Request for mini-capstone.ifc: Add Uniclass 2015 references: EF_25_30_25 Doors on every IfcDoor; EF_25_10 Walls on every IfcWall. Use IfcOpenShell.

First a look at what the model holds.

```python
import ifcopenshell

model = ifcopenshell.open("mini-capstone.ifc")
print(model.schema)
print("classifications:", [c.Name for c in model.by_type("IfcClassification")])
for ifc_class in ("IfcDoor", "IfcRoof", "IfcStair", "IfcWall", "IfcWindow"):
    print(ifc_class, len(model.by_type(ifc_class)))
```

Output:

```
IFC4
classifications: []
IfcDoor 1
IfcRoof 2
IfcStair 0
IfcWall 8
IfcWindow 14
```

```python
import ifcopenshell
import ifcopenshell.api.classification

model = ifcopenshell.open("mini-capstone.ifc")

system = ifcopenshell.api.classification.add_classification(model, classification="Uniclass 2015")

codes = {
    "IfcDoor": ("EF_25_30_25", "Doors"),
    "IfcWall": ("EF_25_10", "Walls"),
}
for ifc_class, (code, name) in codes.items():
    products = model.by_type(ifc_class)
    ifcopenshell.api.classification.add_reference(
        model, products=products, classification=system, identification=code, name=name
    )
    print(code, len(products))

model.write("mini-capstone_updated.ifc")
```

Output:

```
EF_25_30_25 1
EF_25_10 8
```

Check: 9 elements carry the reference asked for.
